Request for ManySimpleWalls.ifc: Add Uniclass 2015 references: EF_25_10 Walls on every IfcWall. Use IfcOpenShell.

First a look at what the model holds.

```python
import ifcopenshell

model = ifcopenshell.open("ManySimpleWalls.ifc")
print(model.schema)
print("classifications:", [c.Name for c in model.by_type("IfcClassification")])
for ifc_class in ("IfcDoor", "IfcRoof", "IfcStair", "IfcWall", "IfcWindow"):
    print(ifc_class, len(model.by_type(ifc_class)))
```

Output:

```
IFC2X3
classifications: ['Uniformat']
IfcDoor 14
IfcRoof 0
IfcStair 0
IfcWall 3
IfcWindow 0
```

```python
import ifcopenshell
import ifcopenshell.api.classification

model = ifcopenshell.open("ManySimpleWalls.ifc")

# IFC2X3 requires Source and Edition and has no link from the project to the system.
system = model.create_entity("IfcClassification", Source="NBS", Edition="2015", Name="Uniclass 2015")

codes = {
    "IfcWall": ("EF_25_10", "Walls"),
}
for ifc_class, (code, name) in codes.items():
    products = model.by_type(ifc_class)
    ifcopenshell.api.classification.add_reference(
        model, products=products, classification=system, identification=code, name=name
    )
    print(code, len(products))

model.write("ManySimpleWalls_v2.ifc")
```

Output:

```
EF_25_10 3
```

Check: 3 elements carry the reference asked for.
